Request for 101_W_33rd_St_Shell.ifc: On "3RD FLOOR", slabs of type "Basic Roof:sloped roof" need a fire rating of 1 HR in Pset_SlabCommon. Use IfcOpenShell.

First a look at what the model holds.

```python
import ifcopenshell
import ifcopenshell.util.element

model = ifcopenshell.open("101_W_33rd_St_Shell.ifc")
print(model.schema)
storey = next(s for s in model.by_type("IfcBuildingStorey") if s.Name == "3RD FLOOR")
slabs = [e for e in ifcopenshell.util.element.get_decomposition(storey) if e.is_a("IfcSlab")]
seen = {}
for e in slabs:
    element_type = ifcopenshell.util.element.get_type(e)
    key = (element_type.Name if element_type != e and element_type else None, ifcopenshell.util.element.get_pset(e, "Pset_SlabCommon", "FireRating"))
    seen[key] = seen.get(key, 0) + 1
for (name, value), count in sorted(seen.items(), key=str):
    print(count, "x", name, "|", value)
```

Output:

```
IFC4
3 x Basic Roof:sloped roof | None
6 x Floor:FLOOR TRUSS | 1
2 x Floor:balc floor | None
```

```python
import ifcopenshell
import ifcopenshell.api.pset
import ifcopenshell.util.element

model = ifcopenshell.open("101_W_33rd_St_Shell.ifc")

storey = next(s for s in model.by_type("IfcBuildingStorey") if s.Name == "3RD FLOOR")
slabs = [e for e in ifcopenshell.util.element.get_decomposition(storey) if e.is_a("IfcSlab")]

count = 0
for e in slabs:
    element_type = ifcopenshell.util.element.get_type(e)
    if element_type in (None, e) or element_type.Name != "Basic Roof:sloped roof":
        continue
    # add_pset returns the element's existing set when there is one.
    pset = ifcopenshell.api.pset.add_pset(model, product=e, name="Pset_SlabCommon")
    ifcopenshell.api.pset.edit_pset(model, pset=pset, properties={"FireRating": "1 HR"})
    count += 1

print(count, "slabs updated")

model.write("101_W_33rd_St_Shell_edited.ifc")
```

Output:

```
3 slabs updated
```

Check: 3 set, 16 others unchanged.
